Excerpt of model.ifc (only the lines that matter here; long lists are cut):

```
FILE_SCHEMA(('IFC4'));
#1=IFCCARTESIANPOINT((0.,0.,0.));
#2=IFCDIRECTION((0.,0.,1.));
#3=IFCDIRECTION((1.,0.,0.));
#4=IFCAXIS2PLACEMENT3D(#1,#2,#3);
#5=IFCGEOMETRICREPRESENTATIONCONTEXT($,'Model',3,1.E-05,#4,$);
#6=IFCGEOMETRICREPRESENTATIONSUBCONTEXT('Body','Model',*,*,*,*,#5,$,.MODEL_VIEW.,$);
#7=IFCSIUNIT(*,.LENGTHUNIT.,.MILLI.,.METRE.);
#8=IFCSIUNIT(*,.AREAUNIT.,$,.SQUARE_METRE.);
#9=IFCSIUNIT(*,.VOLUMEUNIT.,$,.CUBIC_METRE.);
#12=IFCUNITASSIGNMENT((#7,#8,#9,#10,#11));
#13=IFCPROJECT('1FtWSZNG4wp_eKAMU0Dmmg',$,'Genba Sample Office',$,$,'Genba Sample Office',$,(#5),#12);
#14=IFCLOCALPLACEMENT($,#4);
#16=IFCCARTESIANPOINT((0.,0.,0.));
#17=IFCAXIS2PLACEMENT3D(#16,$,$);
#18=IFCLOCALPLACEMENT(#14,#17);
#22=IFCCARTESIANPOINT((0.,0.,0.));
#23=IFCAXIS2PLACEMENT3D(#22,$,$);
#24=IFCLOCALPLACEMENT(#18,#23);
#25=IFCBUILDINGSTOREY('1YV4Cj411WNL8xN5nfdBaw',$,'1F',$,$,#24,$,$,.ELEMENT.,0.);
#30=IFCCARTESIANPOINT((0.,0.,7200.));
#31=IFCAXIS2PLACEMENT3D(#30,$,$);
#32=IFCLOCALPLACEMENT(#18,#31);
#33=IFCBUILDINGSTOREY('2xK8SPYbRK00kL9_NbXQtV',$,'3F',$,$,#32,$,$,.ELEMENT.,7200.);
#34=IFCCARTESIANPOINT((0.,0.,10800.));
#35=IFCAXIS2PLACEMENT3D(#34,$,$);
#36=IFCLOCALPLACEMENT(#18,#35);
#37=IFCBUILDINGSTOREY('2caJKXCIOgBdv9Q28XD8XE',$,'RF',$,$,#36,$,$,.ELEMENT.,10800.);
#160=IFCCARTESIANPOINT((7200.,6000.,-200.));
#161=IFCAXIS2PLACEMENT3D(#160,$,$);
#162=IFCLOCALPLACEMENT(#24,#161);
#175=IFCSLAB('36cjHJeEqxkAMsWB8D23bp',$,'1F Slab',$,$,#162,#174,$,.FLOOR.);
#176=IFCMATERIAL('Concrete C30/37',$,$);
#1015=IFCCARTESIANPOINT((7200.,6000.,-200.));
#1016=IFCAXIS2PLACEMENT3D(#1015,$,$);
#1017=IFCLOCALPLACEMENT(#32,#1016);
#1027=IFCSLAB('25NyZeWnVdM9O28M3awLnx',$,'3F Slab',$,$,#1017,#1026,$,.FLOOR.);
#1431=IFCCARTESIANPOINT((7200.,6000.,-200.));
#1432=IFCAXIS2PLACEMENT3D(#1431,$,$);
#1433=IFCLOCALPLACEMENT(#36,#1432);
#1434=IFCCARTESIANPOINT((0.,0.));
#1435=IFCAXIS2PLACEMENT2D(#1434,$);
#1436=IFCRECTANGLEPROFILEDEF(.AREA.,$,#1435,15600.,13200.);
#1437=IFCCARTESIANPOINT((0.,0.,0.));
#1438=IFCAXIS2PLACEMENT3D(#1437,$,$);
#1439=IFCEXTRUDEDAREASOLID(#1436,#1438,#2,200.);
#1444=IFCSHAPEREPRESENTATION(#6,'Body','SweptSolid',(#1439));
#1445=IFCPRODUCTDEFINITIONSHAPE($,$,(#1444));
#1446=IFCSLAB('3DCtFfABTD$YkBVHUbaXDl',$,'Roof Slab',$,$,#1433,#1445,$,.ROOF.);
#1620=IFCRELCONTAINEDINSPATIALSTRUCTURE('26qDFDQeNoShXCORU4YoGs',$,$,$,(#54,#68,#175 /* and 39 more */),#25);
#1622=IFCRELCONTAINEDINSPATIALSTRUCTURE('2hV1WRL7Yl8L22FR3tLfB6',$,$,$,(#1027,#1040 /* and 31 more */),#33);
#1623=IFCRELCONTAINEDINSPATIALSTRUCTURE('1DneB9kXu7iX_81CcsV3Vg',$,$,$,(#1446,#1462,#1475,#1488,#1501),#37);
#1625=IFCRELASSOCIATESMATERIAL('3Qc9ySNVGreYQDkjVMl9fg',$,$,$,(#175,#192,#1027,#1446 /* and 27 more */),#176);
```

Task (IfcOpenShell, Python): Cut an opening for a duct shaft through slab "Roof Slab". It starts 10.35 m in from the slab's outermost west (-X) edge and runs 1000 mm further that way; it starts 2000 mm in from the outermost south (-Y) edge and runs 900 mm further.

```python
import numpy as np
import ifcopenshell
import ifcopenshell.api.feature
import ifcopenshell.api.geometry
import ifcopenshell.api.root
import ifcopenshell.geom
import ifcopenshell.util.placement
import ifcopenshell.util.representation
import ifcopenshell.util.shape
import ifcopenshell.util.unit

model = ifcopenshell.open("model.ifc")
unit_scale = ifcopenshell.util.unit.calculate_unit_scale(model)
settings = ifcopenshell.geom.settings()


def volume(element):
    """Net volume in cubic metres, openings subtracted."""
    shape = ifcopenshell.geom.create_shape(settings, element)
    return ifcopenshell.util.shape.get_volume(shape.geometry)


slab = model.by_guid("3DCtFfABTD$YkBVHUbaXDl")
before = volume(slab)

# Extent in the slab's own axes, in metres. The edges named are its -X and -Y sides.
slab_shape = ifcopenshell.geom.create_shape(settings, slab)
vertices = ifcopenshell.util.shape.get_vertices(slab_shape.geometry)
x_min, y_min, bottom = vertices.min(axis=0)
top = vertices[:, 2].max()

opening = ifcopenshell.api.root.create_entity(model, ifc_class="IfcOpeningElement", name="Duct shaft opening", predefined_type="OPENING")
context = ifcopenshell.util.representation.get_context(model, "Model", "Body", "MODEL_VIEW")
width, depth = 1, 0.9
outline = [(0.0, 0.0), (width, 0.0), (width, depth), (0.0, depth), (0.0, 0.0)]
# Overshoot both faces by 50 mm so the cut is clean.
shape = ifcopenshell.api.geometry.add_slab_representation(
    model, context=context, depth=top - bottom + 0.1, polyline=outline
)
ifcopenshell.api.geometry.assign_representation(model, product=opening, representation=shape)

matrix = ifcopenshell.util.placement.get_local_placement(slab.ObjectPlacement)
matrix[:, 3] = matrix @ np.append(np.array([x_min + 10.35, y_min + 2, bottom - 0.05]) / unit_scale, 1.0)
ifcopenshell.api.geometry.edit_object_placement(model, product=opening, matrix=matrix, is_si=False)
ifcopenshell.api.feature.add_feature(model, feature=opening, element=slab)

after = volume(slab)

print(f"slab volume {before:.3f} -> {after:.3f} m3")

model.write("model_edited.ifc")
```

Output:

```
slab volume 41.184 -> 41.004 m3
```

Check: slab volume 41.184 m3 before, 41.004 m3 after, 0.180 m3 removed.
